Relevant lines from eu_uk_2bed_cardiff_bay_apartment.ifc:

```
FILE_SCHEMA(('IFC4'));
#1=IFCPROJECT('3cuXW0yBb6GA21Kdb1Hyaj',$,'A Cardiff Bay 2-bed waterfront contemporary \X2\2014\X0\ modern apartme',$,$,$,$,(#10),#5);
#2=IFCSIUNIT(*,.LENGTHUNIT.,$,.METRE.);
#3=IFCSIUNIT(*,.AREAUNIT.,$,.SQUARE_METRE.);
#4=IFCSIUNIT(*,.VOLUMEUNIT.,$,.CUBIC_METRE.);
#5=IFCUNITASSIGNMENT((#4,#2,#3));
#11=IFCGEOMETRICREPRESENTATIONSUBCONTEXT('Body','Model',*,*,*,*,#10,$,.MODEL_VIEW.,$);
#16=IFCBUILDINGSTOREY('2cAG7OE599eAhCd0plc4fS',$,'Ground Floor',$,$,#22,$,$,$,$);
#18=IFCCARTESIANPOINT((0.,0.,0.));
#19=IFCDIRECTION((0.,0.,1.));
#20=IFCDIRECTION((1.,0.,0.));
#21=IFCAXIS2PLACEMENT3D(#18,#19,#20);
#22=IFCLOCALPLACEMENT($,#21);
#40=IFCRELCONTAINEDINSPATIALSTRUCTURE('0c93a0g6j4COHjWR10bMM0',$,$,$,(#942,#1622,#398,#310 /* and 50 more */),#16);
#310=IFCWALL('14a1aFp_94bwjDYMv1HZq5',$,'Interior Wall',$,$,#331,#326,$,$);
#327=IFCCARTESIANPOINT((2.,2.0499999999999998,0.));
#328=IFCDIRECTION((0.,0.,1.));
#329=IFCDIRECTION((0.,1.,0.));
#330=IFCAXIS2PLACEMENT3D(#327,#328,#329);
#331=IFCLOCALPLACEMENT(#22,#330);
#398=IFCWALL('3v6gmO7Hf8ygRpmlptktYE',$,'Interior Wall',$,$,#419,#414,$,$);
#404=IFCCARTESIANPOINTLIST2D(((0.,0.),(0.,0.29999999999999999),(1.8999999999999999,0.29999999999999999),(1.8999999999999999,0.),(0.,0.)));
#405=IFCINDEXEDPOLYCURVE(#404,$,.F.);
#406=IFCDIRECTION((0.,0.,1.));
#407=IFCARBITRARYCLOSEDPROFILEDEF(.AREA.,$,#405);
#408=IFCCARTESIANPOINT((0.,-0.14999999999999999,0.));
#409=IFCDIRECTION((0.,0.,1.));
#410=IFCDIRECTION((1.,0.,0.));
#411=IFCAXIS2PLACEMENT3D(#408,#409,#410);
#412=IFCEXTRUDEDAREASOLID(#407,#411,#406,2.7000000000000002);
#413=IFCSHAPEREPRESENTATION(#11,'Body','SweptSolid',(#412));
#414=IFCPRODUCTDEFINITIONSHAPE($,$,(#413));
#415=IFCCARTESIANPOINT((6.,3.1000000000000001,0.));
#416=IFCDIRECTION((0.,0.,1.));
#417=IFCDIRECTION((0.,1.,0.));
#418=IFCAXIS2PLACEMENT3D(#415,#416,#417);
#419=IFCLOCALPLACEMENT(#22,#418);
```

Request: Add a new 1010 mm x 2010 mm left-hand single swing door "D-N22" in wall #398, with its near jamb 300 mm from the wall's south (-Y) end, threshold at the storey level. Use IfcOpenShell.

```python
import numpy as np
import ifcopenshell
import ifcopenshell.api.feature
import ifcopenshell.api.geometry
import ifcopenshell.api.root
import ifcopenshell.api.spatial
import ifcopenshell.geom
import ifcopenshell.util.element
import ifcopenshell.util.placement
import ifcopenshell.util.representation
import ifcopenshell.util.shape
import ifcopenshell.util.unit

model = ifcopenshell.open("eu_uk_2bed_cardiff_bay_apartment.ifc")
unit_scale = ifcopenshell.util.unit.calculate_unit_scale(model)
settings = ifcopenshell.geom.settings()


def volume(element):
    """Net volume in cubic metres, openings subtracted."""
    shape = ifcopenshell.geom.create_shape(settings, element)
    return ifcopenshell.util.shape.get_volume(shape.geometry)


wall = model.by_guid("3v6gmO7Hf8ygRpmlptktYE")
storey = ifcopenshell.util.element.get_container(wall, ifc_class="IfcBuildingStorey")
context = ifcopenshell.util.representation.get_context(model, "Model", "Body", "MODEL_VIEW")
before = volume(wall)

width, height, from_end, sill = 1.01, 2.01, 0.3, 0.0  # metres

# The wall runs along its own X axis, and the end named is its -X end.
wall_shape = ifcopenshell.geom.create_shape(settings, wall)
x, y, z = ifcopenshell.util.shape.get_vertices(wall_shape.geometry).T
start = x.min() + from_end
face, thickness = float(y.min()), float(y.max() - y.min())
wall_matrix = ifcopenshell.util.placement.get_local_placement(wall.ObjectPlacement)
level = ifcopenshell.util.placement.get_local_placement(storey.ObjectPlacement)[2, 3]


def in_wall(x, y):
    """Placement at x, y metres in the wall's axes, at sill height."""
    matrix = wall_matrix.copy()
    matrix[:, 3] = wall_matrix @ np.array([x / unit_scale, y / unit_scale, 0.0, 1.0])
    matrix[2, 3] = level + sill / unit_scale
    return matrix


# Opening: a box that overshoots both wall faces by 50 mm.
opening = ifcopenshell.api.root.create_entity(model, ifc_class="IfcOpeningElement", predefined_type="OPENING")
box = ifcopenshell.api.geometry.add_wall_representation(
    model, context=context, length=width, height=height, thickness=thickness + 0.1
)
ifcopenshell.api.geometry.assign_representation(model, product=opening, representation=box)
ifcopenshell.api.geometry.edit_object_placement(model, product=opening, matrix=in_wall(start, face - 0.05), is_si=False)
ifcopenshell.api.feature.add_feature(model, feature=opening, element=wall)

door = ifcopenshell.api.root.create_entity(model, ifc_class="IfcDoor", name="D-N22", predefined_type="DOOR")
door.OverallWidth, door.OverallHeight = width / unit_scale, height / unit_scale
door.OperationType = "SINGLE_SWING_LEFT"
body = ifcopenshell.api.geometry.add_door_representation(
    model,
    context=context,
    overall_width=door.OverallWidth,
    overall_height=door.OverallHeight,
    operation_type="SINGLE_SWING_LEFT",
    lining_properties={"LiningDepth": thickness / unit_scale, "ThresholdDepth": thickness / unit_scale},
)
ifcopenshell.api.geometry.assign_representation(model, product=door, representation=body)
ifcopenshell.api.spatial.assign_container(model, products=[door], relating_structure=storey)
ifcopenshell.api.feature.add_filling(model, opening=opening, element=door)

# The lining spans the wall, so the door starts at the wall face.
ifcopenshell.api.geometry.edit_object_placement(model, product=door, matrix=in_wall(start, face), is_si=False)

after = volume(wall)

print(f"wall volume {before:.3f} -> {after:.3f} m3")

model.write("eu_uk_2bed_cardiff_bay_apartment-out.ifc")
```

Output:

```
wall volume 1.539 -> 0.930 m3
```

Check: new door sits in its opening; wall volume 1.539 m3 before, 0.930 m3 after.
